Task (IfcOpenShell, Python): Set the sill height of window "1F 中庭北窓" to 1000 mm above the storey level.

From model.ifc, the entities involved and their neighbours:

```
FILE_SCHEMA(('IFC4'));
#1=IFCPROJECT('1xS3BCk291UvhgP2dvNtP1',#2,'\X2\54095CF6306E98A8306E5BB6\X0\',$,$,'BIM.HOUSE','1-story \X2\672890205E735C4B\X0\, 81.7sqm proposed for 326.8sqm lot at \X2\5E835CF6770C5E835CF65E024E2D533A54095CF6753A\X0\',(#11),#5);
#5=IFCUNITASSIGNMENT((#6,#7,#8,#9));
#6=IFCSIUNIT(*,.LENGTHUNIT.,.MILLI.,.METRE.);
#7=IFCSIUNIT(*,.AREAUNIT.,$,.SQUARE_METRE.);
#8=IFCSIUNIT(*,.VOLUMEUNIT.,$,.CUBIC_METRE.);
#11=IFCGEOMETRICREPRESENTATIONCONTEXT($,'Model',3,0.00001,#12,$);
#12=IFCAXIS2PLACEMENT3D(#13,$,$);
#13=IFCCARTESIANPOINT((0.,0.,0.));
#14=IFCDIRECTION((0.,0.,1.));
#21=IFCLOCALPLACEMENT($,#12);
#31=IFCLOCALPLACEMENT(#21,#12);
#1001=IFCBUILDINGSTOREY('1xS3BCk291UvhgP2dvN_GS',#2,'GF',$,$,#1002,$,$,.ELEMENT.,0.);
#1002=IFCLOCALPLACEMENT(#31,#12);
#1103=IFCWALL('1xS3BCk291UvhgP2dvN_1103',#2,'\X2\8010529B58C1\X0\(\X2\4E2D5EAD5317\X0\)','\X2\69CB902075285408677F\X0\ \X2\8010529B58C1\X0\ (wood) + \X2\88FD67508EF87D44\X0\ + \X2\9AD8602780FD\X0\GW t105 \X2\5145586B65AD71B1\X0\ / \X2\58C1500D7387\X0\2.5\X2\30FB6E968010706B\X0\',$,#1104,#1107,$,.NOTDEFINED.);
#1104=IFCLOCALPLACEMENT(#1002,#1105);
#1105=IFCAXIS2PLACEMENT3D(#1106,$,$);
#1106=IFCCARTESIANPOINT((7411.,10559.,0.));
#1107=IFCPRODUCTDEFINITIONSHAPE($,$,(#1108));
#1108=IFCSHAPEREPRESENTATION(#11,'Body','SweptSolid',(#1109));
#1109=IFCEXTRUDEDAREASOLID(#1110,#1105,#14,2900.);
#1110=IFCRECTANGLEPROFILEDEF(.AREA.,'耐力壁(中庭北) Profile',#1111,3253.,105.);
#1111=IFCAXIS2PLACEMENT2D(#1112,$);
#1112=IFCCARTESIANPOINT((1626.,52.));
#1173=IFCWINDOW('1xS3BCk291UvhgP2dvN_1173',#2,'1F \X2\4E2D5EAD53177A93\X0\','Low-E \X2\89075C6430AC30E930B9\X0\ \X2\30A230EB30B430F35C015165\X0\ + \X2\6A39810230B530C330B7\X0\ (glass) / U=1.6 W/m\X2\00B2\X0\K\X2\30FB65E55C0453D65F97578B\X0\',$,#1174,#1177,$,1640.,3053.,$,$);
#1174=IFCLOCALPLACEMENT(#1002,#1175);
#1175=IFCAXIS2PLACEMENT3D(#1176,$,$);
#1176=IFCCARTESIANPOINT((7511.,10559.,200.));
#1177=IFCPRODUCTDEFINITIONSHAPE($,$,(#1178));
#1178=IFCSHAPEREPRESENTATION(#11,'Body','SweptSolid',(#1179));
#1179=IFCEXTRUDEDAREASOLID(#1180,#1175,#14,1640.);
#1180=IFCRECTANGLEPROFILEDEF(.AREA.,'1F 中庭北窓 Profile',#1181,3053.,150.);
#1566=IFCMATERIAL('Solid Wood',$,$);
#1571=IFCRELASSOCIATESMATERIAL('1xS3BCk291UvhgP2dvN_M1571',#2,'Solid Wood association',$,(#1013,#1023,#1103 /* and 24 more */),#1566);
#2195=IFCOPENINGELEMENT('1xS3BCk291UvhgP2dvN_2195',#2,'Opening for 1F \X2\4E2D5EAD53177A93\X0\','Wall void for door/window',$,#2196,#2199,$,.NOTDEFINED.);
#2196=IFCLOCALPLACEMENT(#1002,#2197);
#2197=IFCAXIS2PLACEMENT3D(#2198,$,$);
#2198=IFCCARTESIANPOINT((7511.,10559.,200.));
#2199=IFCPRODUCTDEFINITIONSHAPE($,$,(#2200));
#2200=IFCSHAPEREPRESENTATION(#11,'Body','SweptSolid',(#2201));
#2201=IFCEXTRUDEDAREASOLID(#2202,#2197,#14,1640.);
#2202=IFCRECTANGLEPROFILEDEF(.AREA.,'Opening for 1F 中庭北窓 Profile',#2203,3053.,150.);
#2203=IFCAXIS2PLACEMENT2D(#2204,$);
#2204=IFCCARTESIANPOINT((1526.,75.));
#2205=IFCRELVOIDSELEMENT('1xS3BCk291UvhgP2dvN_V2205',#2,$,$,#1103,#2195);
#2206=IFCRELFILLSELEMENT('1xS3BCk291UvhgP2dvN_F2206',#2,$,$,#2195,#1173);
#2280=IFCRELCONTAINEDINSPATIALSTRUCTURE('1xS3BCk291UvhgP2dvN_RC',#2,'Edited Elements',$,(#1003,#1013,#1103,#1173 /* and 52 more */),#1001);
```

```python
import numpy as np
import ifcopenshell
import ifcopenshell.api.geometry
import ifcopenshell.geom
import ifcopenshell.util.element
import ifcopenshell.util.placement
import ifcopenshell.util.shape
import ifcopenshell.util.unit

model = ifcopenshell.open("model.ifc")
unit_scale = ifcopenshell.util.unit.calculate_unit_scale(model)

window = model.by_id(1173)
opening = window.FillsVoids[0].RelatingOpeningElement
storey = ifcopenshell.util.element.get_container(window, ifc_class="IfcBuildingStorey")
level = ifcopenshell.util.placement.get_local_placement(storey.ObjectPlacement)[2, 3]

# The opening's origin need not be at the sill, so measure its lowest point.
shape = ifcopenshell.geom.create_shape(ifcopenshell.geom.settings(), opening)
bottom = ifcopenshell.util.shape.get_shape_bottom_elevation(shape, shape.geometry) / unit_scale
dz = level + 1 / unit_scale - bottom

shift = np.array([0.0, 0.0, dz])
# The window is not placed relative to its opening, so move both.
for product in (opening, window):
    matrix = ifcopenshell.util.placement.get_local_placement(product.ObjectPlacement)
    matrix[:3, 3] += shift
    ifcopenshell.api.geometry.edit_object_placement(model, product=product, matrix=matrix, is_si=False)

print(f"moved by {dz * unit_scale:+.3f} m")

model.write("model_edited.ifc")
```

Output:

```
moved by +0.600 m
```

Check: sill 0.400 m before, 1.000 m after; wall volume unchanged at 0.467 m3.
